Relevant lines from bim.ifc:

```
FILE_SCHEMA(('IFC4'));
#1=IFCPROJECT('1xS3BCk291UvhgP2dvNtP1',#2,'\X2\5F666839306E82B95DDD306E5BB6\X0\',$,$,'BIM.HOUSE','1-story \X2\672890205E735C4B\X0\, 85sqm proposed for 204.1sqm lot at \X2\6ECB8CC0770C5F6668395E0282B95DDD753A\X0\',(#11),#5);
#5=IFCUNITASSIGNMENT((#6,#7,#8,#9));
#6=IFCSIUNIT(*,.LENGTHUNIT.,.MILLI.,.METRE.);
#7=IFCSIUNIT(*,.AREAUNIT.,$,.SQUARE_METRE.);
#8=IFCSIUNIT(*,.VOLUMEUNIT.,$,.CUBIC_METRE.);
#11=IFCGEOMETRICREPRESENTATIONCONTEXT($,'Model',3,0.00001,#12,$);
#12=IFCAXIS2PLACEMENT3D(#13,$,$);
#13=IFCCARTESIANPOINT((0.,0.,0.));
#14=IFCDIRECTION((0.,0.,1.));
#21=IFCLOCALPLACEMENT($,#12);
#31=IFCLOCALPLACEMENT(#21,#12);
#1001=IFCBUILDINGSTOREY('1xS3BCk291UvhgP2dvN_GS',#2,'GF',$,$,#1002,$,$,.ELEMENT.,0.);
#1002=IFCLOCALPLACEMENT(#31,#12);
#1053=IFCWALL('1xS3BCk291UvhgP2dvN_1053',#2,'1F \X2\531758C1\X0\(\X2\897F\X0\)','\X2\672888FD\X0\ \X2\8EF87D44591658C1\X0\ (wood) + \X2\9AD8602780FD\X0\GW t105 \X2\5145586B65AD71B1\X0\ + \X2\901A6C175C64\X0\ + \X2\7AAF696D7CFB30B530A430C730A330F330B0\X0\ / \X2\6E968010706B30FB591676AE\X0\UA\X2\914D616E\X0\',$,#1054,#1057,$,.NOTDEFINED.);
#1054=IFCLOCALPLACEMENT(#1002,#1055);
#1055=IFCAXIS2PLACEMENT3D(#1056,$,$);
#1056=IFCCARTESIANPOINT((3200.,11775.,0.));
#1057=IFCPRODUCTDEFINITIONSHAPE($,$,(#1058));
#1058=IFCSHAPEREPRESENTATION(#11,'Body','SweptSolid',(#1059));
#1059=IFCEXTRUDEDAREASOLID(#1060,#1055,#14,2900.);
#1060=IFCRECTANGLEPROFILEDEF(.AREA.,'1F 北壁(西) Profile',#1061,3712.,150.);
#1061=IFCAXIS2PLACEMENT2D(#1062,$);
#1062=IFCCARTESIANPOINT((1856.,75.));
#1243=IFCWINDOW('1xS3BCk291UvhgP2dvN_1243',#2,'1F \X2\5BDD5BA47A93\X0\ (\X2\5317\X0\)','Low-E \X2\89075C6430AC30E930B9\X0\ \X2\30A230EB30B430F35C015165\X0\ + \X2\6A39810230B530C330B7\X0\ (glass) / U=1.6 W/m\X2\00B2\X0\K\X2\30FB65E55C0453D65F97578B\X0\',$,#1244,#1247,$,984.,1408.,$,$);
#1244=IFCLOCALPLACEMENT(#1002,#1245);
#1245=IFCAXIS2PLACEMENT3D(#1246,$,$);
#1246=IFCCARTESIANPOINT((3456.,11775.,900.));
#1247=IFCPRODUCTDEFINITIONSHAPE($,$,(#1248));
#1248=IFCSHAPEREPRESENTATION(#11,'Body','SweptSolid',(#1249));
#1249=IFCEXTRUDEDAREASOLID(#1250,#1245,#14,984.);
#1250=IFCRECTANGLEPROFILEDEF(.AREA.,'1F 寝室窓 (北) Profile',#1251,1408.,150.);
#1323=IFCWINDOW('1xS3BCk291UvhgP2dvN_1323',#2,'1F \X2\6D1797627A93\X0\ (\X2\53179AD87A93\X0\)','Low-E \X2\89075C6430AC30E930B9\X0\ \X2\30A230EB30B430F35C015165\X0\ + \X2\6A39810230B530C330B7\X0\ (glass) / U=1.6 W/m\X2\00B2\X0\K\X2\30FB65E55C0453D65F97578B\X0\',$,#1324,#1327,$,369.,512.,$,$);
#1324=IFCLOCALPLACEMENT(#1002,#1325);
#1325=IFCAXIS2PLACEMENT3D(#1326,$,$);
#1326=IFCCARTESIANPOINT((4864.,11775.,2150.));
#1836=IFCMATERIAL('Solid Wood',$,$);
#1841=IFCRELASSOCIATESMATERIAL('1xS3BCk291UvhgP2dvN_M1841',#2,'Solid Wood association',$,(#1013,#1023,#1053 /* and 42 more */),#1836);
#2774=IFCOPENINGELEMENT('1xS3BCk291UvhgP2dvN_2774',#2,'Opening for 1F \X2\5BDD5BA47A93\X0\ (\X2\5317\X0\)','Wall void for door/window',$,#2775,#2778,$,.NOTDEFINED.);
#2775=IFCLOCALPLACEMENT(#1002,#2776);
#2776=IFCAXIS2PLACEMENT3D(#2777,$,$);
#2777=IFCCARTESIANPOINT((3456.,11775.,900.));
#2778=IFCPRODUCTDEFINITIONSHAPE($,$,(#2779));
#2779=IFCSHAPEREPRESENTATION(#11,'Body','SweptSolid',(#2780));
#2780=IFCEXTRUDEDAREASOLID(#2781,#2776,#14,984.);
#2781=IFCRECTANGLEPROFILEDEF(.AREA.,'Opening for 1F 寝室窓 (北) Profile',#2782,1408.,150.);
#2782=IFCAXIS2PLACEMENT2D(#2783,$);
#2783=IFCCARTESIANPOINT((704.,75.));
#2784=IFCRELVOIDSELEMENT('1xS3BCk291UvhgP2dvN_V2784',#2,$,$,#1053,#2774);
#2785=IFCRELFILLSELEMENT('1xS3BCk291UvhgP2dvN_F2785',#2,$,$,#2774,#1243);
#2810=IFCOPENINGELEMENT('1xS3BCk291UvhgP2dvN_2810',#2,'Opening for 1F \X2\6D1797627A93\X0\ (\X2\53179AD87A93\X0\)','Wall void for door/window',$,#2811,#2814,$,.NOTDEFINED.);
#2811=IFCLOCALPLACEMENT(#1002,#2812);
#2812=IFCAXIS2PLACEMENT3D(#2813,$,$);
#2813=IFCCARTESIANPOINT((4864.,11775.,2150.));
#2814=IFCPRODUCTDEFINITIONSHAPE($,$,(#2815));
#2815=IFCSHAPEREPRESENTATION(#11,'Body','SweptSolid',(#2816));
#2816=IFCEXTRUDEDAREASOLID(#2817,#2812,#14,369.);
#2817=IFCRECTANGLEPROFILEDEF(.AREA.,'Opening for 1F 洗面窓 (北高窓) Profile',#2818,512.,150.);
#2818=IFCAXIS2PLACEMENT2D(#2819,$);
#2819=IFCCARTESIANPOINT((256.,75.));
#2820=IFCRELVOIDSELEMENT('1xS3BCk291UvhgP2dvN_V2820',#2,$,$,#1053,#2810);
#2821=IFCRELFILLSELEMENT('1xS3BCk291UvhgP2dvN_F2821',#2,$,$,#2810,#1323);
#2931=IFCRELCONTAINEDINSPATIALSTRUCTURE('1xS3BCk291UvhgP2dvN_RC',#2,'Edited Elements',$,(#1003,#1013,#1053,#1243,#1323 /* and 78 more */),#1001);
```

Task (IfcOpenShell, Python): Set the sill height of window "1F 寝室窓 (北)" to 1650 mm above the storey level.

```python
import numpy as np
import ifcopenshell
import ifcopenshell.api.geometry
import ifcopenshell.geom
import ifcopenshell.util.element
import ifcopenshell.util.placement
import ifcopenshell.util.shape
import ifcopenshell.util.unit

model = ifcopenshell.open("bim.ifc")
unit_scale = ifcopenshell.util.unit.calculate_unit_scale(model)

window = model.by_id(1243)
opening = window.FillsVoids[0].RelatingOpeningElement
storey = ifcopenshell.util.element.get_container(window, ifc_class="IfcBuildingStorey")
level = ifcopenshell.util.placement.get_local_placement(storey.ObjectPlacement)[2, 3]

# The opening's origin need not be at the sill, so measure its lowest point.
shape = ifcopenshell.geom.create_shape(ifcopenshell.geom.settings(), opening)
bottom = ifcopenshell.util.shape.get_shape_bottom_elevation(shape, shape.geometry) / unit_scale
dz = level + 1650.0 - bottom

shift = np.array([0.0, 0.0, dz])
# The window is not placed relative to its opening, so move both.
for product in (opening, window):
    matrix = ifcopenshell.util.placement.get_local_placement(product.ObjectPlacement)
    matrix[:3, 3] += shift
    ifcopenshell.api.geometry.edit_object_placement(model, product=product, matrix=matrix, is_si=False)

print(f"moved by {dz * unit_scale:+.3f} m")

model.write("bim_edited.ifc")
```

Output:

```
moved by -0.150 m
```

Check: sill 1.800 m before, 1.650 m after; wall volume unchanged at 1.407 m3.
